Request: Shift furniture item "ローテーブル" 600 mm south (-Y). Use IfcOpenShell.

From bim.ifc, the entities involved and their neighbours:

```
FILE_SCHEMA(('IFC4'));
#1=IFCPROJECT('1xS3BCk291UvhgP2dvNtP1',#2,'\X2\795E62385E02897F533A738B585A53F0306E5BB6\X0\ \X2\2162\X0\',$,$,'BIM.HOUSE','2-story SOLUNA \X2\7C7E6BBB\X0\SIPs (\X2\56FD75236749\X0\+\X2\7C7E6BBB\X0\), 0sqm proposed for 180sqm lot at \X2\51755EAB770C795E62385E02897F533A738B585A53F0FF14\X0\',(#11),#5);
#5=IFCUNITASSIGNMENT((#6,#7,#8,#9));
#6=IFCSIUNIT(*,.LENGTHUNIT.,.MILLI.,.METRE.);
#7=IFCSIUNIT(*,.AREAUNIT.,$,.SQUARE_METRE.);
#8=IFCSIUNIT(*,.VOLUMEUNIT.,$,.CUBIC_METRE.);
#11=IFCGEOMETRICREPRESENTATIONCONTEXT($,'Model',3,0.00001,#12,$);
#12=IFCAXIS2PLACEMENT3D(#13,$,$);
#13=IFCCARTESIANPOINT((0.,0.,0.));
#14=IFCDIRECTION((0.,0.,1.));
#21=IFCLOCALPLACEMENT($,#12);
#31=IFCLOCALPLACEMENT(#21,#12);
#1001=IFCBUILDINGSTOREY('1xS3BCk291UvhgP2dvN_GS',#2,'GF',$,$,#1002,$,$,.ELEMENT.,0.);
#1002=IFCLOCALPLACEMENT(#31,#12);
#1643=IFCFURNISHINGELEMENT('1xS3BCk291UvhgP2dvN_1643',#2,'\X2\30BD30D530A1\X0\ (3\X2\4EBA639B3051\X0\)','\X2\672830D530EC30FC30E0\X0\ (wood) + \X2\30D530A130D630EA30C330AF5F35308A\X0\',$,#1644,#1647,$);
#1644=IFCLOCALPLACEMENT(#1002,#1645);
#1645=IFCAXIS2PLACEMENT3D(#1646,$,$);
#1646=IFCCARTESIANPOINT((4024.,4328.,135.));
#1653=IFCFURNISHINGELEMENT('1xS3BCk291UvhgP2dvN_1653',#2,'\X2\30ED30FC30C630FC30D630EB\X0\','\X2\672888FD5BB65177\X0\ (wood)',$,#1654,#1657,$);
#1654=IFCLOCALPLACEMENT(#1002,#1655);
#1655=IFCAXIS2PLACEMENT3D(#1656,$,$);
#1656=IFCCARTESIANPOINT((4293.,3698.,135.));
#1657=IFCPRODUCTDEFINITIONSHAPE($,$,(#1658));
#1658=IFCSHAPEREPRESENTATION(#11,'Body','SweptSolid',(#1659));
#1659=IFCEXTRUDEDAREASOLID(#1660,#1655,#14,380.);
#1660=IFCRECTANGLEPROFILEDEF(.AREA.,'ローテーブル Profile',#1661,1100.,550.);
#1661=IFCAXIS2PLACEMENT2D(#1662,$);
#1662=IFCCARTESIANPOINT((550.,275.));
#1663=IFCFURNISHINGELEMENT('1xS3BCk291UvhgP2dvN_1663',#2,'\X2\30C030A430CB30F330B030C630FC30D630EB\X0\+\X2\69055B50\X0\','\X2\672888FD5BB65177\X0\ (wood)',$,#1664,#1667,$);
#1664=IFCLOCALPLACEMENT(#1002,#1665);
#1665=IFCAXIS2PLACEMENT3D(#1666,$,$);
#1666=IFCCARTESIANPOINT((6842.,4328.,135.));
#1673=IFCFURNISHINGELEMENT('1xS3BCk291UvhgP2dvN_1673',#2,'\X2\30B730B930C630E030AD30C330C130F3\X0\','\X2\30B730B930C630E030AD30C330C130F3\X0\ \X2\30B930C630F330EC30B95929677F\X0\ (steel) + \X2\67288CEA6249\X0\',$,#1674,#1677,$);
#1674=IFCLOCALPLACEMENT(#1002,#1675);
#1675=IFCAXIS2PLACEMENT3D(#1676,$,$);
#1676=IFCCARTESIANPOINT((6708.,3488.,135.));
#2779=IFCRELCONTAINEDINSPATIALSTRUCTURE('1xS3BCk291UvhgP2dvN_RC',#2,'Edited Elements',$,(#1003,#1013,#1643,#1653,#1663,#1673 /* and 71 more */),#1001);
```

```python
import ifcopenshell
import ifcopenshell.api.geometry
import ifcopenshell.util.placement

model = ifcopenshell.open("bim.ifc")

item = model.by_id(1653)
matrix = ifcopenshell.util.placement.get_local_placement(item.ObjectPlacement)
matrix[1, 3] -= 600.0
ifcopenshell.api.geometry.edit_object_placement(model, product=item, matrix=matrix, is_si=False)

print(ifcopenshell.util.placement.get_local_placement(item.ObjectPlacement).round(3) + 0.0)

model.write("bim_edited.ifc")
```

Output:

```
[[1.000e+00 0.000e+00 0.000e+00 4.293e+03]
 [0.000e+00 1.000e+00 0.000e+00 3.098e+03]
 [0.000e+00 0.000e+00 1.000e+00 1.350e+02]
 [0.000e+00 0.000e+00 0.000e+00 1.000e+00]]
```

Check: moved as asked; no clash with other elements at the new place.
